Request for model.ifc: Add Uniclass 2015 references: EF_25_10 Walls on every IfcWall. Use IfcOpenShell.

First a look at what the model holds.

```python
import ifcopenshell

model = ifcopenshell.open("model.ifc")
print(model.schema)
print("classifications:", [c.Name for c in model.by_type("IfcClassification")])
for ifc_class in ("IfcDoor", "IfcRoof", "IfcStair", "IfcWall", "IfcWindow"):
    print(ifc_class, len(model.by_type(ifc_class)))
```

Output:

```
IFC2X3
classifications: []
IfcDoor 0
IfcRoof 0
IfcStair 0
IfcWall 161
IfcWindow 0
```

```python
import ifcopenshell
import ifcopenshell.api.classification

model = ifcopenshell.open("model.ifc")

# IFC2X3 requires Source and Edition and has no link from the project to the system.
system = model.create_entity("IfcClassification", Source="NBS", Edition="2015", Name="Uniclass 2015")

codes = {
    "IfcWall": ("EF_25_10", "Walls"),
}
for ifc_class, (code, name) in codes.items():
    products = model.by_type(ifc_class)
    ifcopenshell.api.classification.add_reference(
        model, products=products, classification=system, identification=code, name=name
    )
    print(code, len(products))

model.write("model_v2.ifc")
```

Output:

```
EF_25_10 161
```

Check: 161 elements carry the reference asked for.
